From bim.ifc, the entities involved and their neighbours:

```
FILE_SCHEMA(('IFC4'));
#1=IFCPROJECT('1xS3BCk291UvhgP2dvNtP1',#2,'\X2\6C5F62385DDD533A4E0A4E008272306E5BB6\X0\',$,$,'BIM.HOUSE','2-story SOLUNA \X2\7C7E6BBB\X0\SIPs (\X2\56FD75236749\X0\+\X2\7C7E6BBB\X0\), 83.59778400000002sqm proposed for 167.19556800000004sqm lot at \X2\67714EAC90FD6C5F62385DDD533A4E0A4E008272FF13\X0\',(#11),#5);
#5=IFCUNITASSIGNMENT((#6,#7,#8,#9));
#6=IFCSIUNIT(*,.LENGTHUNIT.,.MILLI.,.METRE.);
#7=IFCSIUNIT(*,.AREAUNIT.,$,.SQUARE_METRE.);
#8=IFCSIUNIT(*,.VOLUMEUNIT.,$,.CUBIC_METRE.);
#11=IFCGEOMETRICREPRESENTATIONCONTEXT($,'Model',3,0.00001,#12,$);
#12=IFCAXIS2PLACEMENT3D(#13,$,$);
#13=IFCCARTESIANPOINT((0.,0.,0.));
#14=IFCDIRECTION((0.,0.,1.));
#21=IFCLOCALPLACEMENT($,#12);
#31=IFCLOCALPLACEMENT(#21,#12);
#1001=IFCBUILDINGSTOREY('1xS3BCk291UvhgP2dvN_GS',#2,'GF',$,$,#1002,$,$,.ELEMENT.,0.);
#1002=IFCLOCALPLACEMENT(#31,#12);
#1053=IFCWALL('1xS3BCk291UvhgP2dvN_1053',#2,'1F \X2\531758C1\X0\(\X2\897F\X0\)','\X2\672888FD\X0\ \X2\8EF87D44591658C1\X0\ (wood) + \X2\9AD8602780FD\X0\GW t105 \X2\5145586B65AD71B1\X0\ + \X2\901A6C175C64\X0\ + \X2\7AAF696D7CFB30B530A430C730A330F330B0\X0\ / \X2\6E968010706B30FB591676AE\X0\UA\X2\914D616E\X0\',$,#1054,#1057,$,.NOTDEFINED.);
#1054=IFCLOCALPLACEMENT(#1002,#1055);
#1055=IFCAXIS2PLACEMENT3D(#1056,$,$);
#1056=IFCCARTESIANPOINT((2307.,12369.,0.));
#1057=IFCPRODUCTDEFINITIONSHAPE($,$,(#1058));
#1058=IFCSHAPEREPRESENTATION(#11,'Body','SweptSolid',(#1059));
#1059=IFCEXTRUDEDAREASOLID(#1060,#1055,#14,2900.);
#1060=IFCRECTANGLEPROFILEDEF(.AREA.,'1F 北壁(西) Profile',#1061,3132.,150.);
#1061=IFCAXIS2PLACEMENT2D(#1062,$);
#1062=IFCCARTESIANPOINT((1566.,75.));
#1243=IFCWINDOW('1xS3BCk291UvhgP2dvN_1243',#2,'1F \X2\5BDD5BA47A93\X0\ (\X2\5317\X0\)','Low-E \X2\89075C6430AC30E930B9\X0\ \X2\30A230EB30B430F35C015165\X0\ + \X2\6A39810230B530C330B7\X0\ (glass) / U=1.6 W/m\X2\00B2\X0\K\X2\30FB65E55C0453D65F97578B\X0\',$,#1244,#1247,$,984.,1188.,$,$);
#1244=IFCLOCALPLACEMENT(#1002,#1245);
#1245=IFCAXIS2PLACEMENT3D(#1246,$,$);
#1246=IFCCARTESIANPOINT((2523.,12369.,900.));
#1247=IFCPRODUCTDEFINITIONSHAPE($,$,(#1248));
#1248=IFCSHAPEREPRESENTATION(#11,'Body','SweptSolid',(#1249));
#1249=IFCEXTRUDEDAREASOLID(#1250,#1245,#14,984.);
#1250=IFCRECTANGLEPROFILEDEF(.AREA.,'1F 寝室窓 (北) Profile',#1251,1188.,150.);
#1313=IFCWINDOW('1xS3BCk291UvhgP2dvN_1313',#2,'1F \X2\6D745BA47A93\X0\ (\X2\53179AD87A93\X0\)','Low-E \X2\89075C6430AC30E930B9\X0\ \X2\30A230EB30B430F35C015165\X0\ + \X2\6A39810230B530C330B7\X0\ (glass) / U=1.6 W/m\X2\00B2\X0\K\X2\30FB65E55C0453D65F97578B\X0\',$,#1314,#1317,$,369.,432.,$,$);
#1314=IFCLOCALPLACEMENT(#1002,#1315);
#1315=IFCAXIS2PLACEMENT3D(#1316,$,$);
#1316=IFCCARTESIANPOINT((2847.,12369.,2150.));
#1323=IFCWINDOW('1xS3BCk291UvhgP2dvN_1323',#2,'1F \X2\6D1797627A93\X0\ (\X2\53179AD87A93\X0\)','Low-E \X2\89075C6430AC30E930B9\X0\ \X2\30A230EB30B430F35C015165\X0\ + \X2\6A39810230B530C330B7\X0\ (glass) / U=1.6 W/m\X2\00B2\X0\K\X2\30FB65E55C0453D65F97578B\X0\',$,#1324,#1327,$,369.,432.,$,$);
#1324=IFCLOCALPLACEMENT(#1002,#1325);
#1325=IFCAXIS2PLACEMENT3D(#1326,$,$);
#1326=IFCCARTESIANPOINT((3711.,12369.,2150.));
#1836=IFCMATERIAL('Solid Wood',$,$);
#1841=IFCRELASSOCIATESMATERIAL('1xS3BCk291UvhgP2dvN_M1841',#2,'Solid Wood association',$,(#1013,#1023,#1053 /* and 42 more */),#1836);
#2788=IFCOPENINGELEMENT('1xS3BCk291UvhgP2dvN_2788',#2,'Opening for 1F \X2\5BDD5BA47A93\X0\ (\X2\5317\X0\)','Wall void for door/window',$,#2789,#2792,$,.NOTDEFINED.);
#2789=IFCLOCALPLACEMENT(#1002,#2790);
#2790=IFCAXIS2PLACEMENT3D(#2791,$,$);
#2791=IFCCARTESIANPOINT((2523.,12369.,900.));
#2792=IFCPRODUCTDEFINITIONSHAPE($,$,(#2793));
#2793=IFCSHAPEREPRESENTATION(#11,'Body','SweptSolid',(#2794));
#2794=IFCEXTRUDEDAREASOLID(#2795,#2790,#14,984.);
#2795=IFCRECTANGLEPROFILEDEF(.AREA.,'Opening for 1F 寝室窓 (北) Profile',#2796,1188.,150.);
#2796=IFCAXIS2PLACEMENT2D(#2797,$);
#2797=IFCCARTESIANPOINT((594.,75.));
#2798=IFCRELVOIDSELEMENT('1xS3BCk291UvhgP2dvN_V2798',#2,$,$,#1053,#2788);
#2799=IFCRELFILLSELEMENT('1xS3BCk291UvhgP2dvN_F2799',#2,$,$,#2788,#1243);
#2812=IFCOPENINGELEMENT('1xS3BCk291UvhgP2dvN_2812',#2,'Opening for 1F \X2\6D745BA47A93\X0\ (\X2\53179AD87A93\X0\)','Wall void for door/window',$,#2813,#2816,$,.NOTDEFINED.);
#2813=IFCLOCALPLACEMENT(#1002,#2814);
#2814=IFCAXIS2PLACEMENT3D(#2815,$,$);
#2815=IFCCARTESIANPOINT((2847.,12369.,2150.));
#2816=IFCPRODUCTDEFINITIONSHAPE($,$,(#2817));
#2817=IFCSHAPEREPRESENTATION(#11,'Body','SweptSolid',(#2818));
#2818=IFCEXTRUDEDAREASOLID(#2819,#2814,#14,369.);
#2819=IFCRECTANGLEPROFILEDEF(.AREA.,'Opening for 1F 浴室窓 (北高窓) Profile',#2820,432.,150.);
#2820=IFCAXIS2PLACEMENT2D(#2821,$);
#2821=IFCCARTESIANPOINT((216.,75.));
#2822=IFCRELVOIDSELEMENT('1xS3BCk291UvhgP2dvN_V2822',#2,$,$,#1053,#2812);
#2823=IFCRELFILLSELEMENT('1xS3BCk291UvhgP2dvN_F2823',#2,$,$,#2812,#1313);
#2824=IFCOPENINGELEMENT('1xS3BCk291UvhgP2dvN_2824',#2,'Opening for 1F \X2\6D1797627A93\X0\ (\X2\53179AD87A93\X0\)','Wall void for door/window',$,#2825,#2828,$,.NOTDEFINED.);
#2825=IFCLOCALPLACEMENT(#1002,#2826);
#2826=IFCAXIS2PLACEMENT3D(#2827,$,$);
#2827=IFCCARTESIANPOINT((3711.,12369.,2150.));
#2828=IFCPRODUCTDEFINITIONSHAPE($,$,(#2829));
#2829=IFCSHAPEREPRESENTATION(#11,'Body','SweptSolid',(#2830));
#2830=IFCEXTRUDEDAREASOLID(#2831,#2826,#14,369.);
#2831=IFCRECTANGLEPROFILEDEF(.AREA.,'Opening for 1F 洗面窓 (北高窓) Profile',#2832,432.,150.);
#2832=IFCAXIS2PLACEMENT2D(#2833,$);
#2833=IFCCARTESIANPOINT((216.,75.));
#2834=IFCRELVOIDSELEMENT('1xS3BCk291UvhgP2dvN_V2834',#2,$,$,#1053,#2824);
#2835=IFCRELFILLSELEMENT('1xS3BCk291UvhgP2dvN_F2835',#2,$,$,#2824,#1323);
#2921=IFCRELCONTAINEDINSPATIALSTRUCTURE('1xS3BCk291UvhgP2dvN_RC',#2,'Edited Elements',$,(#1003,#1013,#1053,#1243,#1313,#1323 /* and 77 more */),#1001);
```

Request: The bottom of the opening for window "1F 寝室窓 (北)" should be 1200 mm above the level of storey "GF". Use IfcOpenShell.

```python
import numpy as np
import ifcopenshell
import ifcopenshell.api.geometry
import ifcopenshell.geom
import ifcopenshell.util.element
import ifcopenshell.util.placement
import ifcopenshell.util.shape
import ifcopenshell.util.unit

model = ifcopenshell.open("bim.ifc")
unit_scale = ifcopenshell.util.unit.calculate_unit_scale(model)

window = model.by_id(1243)
opening = window.FillsVoids[0].RelatingOpeningElement
storey = ifcopenshell.util.element.get_container(window, ifc_class="IfcBuildingStorey")
level = ifcopenshell.util.placement.get_local_placement(storey.ObjectPlacement)[2, 3]

# The opening's origin need not be at the sill, so measure its lowest point.
shape = ifcopenshell.geom.create_shape(ifcopenshell.geom.settings(), opening)
bottom = ifcopenshell.util.shape.get_shape_bottom_elevation(shape, shape.geometry) / unit_scale
dz = level + 1.2 / unit_scale - bottom

shift = np.array([0.0, 0.0, dz])
# The window is not placed relative to its opening, so move both.
for product in (opening, window):
    matrix = ifcopenshell.util.placement.get_local_placement(product.ObjectPlacement)
    matrix[:3, 3] += shift
    ifcopenshell.api.geometry.edit_object_placement(model, product=product, matrix=matrix, is_si=False)

print(f"moved by {dz * unit_scale:+.3f} m")

model.write("bim_updated.ifc")
```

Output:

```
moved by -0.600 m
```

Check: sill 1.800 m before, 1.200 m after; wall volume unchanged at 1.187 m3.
